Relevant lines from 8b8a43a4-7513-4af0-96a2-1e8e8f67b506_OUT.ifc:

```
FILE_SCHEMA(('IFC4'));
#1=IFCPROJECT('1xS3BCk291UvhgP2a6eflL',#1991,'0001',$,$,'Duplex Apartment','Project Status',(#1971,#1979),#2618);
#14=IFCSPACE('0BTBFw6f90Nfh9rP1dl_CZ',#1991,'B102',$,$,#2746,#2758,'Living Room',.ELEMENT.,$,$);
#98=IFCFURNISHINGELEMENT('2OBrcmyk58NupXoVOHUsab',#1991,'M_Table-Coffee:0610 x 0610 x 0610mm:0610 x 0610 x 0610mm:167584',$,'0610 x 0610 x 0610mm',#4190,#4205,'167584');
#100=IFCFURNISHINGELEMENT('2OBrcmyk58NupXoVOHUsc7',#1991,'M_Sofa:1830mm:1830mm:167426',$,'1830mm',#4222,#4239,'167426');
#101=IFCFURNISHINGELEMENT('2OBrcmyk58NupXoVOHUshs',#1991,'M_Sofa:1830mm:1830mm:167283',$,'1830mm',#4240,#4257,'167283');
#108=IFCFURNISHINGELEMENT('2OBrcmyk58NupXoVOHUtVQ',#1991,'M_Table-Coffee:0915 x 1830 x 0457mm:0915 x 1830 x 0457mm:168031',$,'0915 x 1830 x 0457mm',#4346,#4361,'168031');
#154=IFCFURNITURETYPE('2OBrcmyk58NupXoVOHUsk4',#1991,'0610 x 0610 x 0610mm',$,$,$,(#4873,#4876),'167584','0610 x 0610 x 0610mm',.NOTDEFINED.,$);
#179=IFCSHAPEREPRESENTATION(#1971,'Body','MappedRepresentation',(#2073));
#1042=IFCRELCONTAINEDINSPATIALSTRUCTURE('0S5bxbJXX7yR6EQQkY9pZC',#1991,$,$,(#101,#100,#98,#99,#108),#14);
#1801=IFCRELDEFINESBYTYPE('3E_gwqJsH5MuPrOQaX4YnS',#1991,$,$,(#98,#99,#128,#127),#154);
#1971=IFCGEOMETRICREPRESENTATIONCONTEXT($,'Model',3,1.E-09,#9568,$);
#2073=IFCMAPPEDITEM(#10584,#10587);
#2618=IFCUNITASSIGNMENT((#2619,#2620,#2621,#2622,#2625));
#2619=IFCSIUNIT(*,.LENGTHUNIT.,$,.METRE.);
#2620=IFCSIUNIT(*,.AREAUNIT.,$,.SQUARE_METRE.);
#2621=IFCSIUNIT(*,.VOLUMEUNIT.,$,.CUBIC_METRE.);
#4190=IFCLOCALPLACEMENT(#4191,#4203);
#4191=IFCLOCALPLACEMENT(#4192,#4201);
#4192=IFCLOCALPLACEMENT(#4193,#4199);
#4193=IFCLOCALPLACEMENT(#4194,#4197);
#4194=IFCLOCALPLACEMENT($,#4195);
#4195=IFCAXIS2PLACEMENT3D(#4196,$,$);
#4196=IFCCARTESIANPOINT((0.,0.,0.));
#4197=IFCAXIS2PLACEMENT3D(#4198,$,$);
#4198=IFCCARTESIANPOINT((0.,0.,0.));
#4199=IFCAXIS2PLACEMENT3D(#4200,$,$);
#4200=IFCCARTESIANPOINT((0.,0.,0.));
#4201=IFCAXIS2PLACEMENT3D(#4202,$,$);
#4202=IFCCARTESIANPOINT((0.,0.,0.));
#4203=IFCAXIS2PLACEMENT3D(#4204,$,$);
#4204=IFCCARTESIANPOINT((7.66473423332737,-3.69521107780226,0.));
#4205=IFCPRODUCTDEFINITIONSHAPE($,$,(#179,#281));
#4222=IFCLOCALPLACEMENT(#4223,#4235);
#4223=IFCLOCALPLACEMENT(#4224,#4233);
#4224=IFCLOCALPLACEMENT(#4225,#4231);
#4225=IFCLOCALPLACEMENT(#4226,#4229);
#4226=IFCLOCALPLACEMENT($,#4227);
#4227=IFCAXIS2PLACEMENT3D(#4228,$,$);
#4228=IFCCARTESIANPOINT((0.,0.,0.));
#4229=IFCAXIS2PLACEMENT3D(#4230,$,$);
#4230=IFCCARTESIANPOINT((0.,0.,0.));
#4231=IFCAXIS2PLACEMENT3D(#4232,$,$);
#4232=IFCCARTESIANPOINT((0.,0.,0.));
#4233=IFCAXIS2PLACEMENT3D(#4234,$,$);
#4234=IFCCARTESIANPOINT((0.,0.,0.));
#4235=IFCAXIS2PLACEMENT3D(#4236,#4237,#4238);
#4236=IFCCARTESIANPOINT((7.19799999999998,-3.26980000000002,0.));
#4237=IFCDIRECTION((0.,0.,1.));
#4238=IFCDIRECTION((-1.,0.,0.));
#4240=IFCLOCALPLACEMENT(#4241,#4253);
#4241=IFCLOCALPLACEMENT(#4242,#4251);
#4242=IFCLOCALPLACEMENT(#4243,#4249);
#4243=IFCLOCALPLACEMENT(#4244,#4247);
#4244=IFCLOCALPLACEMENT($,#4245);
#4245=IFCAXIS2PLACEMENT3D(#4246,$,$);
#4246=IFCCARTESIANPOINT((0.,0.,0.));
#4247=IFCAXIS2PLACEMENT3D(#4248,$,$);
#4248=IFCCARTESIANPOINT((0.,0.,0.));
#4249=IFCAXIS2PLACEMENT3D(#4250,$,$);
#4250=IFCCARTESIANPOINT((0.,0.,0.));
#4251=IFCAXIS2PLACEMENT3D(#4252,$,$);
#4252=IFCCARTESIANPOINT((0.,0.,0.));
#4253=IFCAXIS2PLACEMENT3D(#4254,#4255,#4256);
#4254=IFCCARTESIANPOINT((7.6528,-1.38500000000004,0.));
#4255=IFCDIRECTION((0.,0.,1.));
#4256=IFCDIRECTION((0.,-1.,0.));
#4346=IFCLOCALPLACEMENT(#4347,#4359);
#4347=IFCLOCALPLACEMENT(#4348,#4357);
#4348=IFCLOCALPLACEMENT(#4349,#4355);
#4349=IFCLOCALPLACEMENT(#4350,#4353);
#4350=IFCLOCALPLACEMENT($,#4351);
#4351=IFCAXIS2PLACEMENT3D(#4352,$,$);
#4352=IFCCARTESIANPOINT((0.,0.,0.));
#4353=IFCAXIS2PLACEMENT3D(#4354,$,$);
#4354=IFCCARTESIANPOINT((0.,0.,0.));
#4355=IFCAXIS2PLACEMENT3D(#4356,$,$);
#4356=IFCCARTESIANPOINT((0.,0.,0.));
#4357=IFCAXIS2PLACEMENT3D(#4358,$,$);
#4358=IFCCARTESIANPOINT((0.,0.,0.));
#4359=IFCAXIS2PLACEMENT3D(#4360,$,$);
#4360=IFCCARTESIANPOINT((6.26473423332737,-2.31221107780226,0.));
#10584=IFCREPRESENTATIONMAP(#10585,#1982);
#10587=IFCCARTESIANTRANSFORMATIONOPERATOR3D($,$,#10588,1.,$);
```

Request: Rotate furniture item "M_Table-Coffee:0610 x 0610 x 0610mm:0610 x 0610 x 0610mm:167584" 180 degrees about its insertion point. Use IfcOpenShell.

```python
import ifcopenshell
import ifcopenshell.api.geometry
import ifcopenshell.util.placement

model = ifcopenshell.open("8b8a43a4-7513-4af0-96a2-1e8e8f67b506_OUT.ifc")

item = model.by_id(98)
matrix = ifcopenshell.util.placement.get_local_placement(item.ObjectPlacement)
matrix = matrix @ ifcopenshell.util.placement.rotation(180, "Z")
ifcopenshell.api.geometry.edit_object_placement(model, product=item, matrix=matrix, is_si=False)

print(ifcopenshell.util.placement.get_local_placement(item.ObjectPlacement).round(3) + 0.0)

model.write("8b8a43a4-7513-4af0-96a2-1e8e8f67b506_OUT_rev.ifc")
```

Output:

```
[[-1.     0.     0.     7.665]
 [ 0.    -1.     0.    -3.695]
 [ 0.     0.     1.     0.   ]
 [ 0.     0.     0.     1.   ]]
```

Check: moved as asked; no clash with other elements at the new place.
